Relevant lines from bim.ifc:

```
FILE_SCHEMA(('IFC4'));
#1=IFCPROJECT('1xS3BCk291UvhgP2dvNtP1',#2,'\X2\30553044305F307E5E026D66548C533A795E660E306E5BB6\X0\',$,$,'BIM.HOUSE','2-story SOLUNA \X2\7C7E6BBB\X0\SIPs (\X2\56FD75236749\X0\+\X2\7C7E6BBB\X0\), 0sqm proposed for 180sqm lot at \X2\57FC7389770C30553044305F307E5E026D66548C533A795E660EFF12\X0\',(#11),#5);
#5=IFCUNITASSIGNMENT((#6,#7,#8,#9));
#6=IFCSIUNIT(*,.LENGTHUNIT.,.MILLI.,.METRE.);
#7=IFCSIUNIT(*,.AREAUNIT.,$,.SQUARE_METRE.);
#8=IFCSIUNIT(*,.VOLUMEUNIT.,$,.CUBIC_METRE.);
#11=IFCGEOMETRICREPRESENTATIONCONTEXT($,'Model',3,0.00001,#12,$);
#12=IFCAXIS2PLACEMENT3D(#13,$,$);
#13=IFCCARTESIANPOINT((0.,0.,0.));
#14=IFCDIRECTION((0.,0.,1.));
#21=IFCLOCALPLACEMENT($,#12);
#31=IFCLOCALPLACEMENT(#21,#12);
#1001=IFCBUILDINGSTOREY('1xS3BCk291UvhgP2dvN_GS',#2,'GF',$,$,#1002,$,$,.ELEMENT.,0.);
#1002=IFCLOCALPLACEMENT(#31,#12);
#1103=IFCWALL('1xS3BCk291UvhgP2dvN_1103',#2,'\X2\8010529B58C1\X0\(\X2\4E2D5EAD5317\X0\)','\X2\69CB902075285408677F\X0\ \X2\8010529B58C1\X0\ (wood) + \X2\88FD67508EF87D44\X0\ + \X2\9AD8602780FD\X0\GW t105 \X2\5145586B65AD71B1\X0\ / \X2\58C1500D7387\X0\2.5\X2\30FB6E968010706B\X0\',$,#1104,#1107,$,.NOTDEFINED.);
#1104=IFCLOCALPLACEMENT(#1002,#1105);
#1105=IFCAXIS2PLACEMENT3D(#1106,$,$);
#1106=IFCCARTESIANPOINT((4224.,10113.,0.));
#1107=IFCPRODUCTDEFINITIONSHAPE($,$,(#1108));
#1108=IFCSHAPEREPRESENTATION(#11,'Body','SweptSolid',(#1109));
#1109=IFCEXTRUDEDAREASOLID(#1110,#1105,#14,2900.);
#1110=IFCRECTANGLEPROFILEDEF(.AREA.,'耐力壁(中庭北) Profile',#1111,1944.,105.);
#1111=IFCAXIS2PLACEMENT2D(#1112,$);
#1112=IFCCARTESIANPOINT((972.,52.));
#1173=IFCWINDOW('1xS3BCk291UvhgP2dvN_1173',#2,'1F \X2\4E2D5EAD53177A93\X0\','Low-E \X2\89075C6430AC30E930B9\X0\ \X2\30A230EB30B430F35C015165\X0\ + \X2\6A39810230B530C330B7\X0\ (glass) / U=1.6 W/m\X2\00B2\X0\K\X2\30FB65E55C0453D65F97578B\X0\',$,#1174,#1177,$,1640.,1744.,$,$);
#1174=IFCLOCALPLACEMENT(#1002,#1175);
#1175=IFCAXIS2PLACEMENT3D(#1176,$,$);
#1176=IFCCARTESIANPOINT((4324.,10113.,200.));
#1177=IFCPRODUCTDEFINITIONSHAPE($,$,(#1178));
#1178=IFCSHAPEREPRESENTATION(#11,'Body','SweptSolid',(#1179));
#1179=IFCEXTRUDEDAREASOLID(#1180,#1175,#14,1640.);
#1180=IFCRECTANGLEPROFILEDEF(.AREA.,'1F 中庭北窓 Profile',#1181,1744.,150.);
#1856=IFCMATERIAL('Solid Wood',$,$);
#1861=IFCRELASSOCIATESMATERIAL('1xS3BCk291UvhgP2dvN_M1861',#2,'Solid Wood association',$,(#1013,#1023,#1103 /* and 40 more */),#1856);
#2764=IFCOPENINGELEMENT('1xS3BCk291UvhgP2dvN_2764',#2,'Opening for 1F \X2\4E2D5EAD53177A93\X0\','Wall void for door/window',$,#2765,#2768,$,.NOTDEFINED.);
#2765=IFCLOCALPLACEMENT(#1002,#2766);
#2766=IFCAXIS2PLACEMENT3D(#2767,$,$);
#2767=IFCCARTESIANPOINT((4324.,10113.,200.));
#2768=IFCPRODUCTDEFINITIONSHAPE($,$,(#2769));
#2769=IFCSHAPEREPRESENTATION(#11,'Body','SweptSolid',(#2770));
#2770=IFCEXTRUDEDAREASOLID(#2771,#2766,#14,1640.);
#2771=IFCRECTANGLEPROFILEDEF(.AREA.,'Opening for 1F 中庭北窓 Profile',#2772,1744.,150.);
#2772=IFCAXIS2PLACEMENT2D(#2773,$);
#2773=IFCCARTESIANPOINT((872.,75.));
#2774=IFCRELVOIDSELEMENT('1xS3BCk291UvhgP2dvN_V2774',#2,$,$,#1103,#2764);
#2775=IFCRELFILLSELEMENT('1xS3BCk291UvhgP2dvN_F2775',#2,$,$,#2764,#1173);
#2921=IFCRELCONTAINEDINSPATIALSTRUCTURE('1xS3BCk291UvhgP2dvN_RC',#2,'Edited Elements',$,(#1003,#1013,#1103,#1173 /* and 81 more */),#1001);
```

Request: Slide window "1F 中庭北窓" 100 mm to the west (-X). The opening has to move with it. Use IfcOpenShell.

```python
import ifcopenshell
import ifcopenshell.api.geometry
import ifcopenshell.util.placement
import ifcopenshell.util.unit

model = ifcopenshell.open("bim.ifc")
unit_scale = ifcopenshell.util.unit.calculate_unit_scale(model)

window = model.by_guid("1xS3BCk291UvhgP2dvN_1173")
opening = window.FillsVoids[0].RelatingOpeningElement
wall = opening.VoidsElements[0].RelatingBuildingElement

wall_matrix = ifcopenshell.util.placement.get_local_placement(wall.ObjectPlacement)
shift = wall_matrix[:3, 0] * -0.1 / unit_scale
before = ifcopenshell.util.placement.get_local_placement(window.ObjectPlacement)[:3, 3].copy()

# The window is not placed relative to its opening, so move both.
for product in (opening, window):
    matrix = ifcopenshell.util.placement.get_local_placement(product.ObjectPlacement)
    matrix[:3, 3] += shift
    ifcopenshell.api.geometry.edit_object_placement(model, product=product, matrix=matrix, is_si=False)

after = ifcopenshell.util.placement.get_local_placement(window.ObjectPlacement)[:3, 3]
print("window moved by", (after - before).round(3) + 0.0)

model.write("bim_rev.ifc")
```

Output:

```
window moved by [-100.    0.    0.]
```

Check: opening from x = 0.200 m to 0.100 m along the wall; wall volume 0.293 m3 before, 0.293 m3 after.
